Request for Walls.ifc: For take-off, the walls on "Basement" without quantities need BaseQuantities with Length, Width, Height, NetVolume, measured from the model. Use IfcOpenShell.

First a look at what the model holds.

```python
import ifcopenshell
import ifcopenshell.util.element
import ifcopenshell.util.unit

model = ifcopenshell.open("Walls.ifc")
print(model.schema)
for unit_type in ("LENGTHUNIT", "AREAUNIT", "VOLUMEUNIT"):
    print(unit_type, ifcopenshell.util.unit.calculate_unit_scale(model, unit_type))
storey = next(s for s in model.by_type("IfcBuildingStorey") if s.Name == "Basement")
walls = [e for e in ifcopenshell.util.element.get_decomposition(storey) if e.is_a("IfcWall")]
for e in sorted(walls, key=lambda e: e.id()):
    print(e.id(), e.is_a(), e.Name, list(ifcopenshell.util.element.get_psets(e, qtos_only=True)), sep=" | ")
```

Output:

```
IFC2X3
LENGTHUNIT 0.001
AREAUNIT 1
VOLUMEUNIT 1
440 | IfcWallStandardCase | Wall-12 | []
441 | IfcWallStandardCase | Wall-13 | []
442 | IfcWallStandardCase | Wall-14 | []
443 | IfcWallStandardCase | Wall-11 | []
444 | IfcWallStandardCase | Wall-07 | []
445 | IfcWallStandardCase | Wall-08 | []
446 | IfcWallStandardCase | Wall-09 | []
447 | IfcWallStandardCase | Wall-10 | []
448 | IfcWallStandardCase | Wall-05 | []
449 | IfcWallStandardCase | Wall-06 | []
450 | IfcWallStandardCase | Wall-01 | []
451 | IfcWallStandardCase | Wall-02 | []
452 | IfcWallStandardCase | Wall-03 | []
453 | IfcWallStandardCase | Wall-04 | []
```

```python
import ifcopenshell
import ifcopenshell.api.pset
import ifcopenshell.geom
import ifcopenshell.util.element
import ifcopenshell.util.shape
import ifcopenshell.util.unit

model = ifcopenshell.open("Walls.ifc")
unit_scale = ifcopenshell.util.unit.calculate_unit_scale(model)
volume_scale = ifcopenshell.util.unit.calculate_unit_scale(model, "VOLUMEUNIT")
settings = ifcopenshell.geom.settings()

storey = next(s for s in model.by_type("IfcBuildingStorey") if s.Name == "Basement")
walls = [e for e in ifcopenshell.util.element.get_decomposition(storey) if e.is_a("IfcWall")]

for e in sorted(walls, key=lambda e: e.id()):
    if ifcopenshell.util.element.get_psets(e, qtos_only=True, should_inherit=False):
        continue
    # Geometry comes back in metres, in the element's own axes.
    shape = ifcopenshell.geom.create_shape(settings, e)
    values = {
        "Length": ifcopenshell.util.shape.get_x(shape.geometry) / unit_scale,
        "Width": ifcopenshell.util.shape.get_y(shape.geometry) / unit_scale,
        "Height": ifcopenshell.util.shape.get_z(shape.geometry) / unit_scale,
        "NetVolume": ifcopenshell.util.shape.get_volume(shape.geometry) / volume_scale,
    }
    qto = ifcopenshell.api.pset.add_qto(model, product=e, name="BaseQuantities")
    ifcopenshell.api.pset.edit_qto(model, qto=qto, properties=values)
    print(e.id(), {k: round(v, 3) for k, v in values.items()})

model.write("Walls_edited.ifc")
```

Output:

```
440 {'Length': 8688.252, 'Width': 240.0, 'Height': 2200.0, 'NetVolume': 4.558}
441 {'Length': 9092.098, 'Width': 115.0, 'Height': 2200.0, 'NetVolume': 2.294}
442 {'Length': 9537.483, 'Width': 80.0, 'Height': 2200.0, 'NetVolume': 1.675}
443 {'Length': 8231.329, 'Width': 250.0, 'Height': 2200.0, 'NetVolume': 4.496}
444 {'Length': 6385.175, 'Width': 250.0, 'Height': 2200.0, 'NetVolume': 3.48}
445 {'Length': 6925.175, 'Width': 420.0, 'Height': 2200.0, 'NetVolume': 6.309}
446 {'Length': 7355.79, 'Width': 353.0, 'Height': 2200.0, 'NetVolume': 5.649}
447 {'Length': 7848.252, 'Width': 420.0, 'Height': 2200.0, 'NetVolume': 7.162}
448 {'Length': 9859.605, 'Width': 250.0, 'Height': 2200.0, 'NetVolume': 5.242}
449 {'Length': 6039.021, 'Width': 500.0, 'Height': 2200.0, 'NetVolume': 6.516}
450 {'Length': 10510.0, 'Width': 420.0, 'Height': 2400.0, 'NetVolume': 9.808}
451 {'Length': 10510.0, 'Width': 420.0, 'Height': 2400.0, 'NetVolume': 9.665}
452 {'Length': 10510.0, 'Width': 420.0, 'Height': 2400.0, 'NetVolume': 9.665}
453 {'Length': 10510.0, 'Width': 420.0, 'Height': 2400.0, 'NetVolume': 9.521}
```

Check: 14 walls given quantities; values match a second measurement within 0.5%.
